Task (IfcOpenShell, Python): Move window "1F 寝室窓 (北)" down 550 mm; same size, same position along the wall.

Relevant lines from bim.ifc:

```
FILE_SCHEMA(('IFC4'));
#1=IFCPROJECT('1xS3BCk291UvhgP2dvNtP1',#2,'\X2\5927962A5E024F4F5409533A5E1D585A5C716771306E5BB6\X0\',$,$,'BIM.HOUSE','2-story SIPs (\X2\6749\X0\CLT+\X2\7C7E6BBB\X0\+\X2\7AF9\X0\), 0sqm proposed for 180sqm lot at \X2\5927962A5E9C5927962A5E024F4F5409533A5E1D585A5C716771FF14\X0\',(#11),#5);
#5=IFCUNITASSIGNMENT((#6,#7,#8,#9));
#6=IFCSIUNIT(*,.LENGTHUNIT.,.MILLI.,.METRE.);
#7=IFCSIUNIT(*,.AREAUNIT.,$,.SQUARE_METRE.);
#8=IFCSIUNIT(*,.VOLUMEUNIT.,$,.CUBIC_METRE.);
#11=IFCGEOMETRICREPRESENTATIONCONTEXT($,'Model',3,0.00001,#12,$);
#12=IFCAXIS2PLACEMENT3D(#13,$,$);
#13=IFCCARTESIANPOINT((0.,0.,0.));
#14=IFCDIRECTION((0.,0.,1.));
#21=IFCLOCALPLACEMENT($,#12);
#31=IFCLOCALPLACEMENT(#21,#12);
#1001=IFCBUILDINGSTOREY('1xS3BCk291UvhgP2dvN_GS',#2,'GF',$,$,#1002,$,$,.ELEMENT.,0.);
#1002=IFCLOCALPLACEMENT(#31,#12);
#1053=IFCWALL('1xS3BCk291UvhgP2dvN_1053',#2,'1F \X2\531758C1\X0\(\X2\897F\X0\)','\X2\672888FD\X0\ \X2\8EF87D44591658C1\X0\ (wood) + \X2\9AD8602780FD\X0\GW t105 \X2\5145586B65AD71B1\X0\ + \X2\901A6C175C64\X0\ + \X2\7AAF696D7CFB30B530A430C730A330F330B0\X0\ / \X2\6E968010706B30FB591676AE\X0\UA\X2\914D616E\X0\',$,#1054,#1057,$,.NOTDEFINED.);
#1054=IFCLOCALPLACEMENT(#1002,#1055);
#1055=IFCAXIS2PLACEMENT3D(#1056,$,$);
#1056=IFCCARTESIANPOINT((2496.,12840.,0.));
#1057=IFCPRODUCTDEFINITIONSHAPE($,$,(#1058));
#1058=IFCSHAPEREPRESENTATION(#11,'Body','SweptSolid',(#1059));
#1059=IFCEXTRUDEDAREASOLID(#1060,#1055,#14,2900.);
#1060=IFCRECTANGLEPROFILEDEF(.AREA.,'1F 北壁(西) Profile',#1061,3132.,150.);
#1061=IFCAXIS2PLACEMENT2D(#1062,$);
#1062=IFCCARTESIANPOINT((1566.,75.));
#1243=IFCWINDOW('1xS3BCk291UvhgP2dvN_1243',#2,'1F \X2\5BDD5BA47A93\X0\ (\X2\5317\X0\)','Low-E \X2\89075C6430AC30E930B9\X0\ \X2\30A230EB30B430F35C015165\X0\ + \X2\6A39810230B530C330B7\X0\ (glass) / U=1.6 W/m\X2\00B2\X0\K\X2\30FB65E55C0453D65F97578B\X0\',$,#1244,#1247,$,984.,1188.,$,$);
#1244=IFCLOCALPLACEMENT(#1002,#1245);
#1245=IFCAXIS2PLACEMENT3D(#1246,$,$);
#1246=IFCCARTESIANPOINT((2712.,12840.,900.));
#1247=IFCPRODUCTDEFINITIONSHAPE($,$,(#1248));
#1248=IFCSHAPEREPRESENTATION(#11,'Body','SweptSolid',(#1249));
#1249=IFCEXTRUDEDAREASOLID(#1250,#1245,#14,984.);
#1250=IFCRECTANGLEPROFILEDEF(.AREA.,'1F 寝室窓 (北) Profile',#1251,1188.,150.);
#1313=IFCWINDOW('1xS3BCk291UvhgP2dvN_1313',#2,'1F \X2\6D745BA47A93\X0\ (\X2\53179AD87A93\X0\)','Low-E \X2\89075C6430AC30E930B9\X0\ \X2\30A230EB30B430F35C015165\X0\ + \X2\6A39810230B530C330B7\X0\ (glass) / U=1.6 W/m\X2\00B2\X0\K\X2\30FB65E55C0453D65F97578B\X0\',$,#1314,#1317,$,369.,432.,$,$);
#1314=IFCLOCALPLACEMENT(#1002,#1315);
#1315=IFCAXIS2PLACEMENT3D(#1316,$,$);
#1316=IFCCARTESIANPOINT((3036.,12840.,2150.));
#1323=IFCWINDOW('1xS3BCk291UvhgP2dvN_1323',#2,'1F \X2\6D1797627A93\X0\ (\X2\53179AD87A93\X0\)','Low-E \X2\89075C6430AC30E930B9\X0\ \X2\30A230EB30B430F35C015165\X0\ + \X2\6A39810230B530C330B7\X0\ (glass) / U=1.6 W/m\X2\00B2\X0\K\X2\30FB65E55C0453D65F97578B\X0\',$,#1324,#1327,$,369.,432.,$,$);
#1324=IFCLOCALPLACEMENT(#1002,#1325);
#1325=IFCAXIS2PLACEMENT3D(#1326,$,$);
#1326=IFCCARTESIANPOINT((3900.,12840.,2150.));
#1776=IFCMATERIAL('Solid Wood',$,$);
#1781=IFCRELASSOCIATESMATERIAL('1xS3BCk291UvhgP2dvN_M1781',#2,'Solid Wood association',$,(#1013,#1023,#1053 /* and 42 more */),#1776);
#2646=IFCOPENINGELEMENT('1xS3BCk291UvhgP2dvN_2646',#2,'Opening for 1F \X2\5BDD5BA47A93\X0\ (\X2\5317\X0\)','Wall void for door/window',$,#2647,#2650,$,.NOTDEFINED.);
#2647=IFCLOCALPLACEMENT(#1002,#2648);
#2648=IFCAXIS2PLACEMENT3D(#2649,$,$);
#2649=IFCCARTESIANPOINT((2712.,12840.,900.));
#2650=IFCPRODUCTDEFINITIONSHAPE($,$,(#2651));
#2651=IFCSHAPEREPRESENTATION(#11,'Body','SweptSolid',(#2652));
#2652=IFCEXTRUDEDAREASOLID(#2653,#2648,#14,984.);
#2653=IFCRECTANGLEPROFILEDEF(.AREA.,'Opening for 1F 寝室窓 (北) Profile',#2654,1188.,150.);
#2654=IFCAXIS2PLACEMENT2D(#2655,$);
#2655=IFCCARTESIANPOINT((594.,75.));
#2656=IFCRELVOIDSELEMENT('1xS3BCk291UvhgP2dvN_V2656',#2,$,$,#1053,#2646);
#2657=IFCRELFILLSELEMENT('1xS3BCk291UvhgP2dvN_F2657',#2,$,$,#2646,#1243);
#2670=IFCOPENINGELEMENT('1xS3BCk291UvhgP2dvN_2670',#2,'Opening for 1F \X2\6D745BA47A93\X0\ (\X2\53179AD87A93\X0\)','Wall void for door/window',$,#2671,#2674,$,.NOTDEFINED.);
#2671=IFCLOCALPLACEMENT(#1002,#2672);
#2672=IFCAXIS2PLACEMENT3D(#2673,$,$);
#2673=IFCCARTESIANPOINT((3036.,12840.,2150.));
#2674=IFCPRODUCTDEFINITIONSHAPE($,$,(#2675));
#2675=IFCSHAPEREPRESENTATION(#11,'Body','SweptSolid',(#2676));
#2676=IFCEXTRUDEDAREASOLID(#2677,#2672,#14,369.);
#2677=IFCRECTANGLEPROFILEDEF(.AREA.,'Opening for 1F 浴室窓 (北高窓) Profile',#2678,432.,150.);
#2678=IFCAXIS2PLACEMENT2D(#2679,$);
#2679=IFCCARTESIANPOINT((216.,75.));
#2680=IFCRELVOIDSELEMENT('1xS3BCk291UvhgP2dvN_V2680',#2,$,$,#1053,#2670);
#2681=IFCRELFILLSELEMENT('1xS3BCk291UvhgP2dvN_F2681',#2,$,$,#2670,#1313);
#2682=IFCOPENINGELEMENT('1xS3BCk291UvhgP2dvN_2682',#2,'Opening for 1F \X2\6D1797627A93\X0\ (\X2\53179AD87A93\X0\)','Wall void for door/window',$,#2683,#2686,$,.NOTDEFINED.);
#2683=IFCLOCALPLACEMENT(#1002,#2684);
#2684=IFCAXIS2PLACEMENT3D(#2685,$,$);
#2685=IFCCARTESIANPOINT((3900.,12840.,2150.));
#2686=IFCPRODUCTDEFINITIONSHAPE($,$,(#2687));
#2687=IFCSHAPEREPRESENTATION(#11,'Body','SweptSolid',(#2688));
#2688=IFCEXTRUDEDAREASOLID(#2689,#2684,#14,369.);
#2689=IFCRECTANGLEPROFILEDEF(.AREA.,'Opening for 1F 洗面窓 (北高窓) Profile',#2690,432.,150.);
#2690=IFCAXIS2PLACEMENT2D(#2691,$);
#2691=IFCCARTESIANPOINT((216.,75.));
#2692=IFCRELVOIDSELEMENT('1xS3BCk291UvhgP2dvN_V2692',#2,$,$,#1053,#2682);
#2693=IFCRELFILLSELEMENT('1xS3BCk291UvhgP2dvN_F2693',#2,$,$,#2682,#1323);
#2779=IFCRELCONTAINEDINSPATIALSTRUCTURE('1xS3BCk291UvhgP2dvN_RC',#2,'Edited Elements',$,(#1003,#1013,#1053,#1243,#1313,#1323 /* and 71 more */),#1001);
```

```python
import numpy as np
import ifcopenshell
import ifcopenshell.api.geometry
import ifcopenshell.util.placement
import ifcopenshell.util.unit

model = ifcopenshell.open("bim.ifc")
unit_scale = ifcopenshell.util.unit.calculate_unit_scale(model)

window = model.by_guid("1xS3BCk291UvhgP2dvN_1243")
opening = window.FillsVoids[0].RelatingOpeningElement
dz = -0.55 / unit_scale

shift = np.array([0.0, 0.0, dz])
# The window is not placed relative to its opening, so move both.
for product in (opening, window):
    matrix = ifcopenshell.util.placement.get_local_placement(product.ObjectPlacement)
    matrix[:3, 3] += shift
    ifcopenshell.api.geometry.edit_object_placement(model, product=product, matrix=matrix, is_si=False)

print(f"moved by {dz * unit_scale:+.3f} m")

model.write("bim_updated.ifc")
```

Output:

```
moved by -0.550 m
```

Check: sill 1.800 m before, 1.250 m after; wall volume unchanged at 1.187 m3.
